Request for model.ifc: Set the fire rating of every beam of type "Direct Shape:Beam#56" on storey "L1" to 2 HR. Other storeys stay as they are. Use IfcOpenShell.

First a look at what the model holds.

```python
import ifcopenshell
import ifcopenshell.util.element

model = ifcopenshell.open("model.ifc")
print(model.schema)
storey = next(s for s in model.by_type("IfcBuildingStorey") if s.Name == "L1")
beams = [e for e in ifcopenshell.util.element.get_decomposition(storey) if e.is_a("IfcBeam")]
seen = {}
for e in beams:
    element_type = ifcopenshell.util.element.get_type(e)
    key = (element_type.Name if element_type != e and element_type else None, ifcopenshell.util.element.get_pset(e, "Pset_BeamCommon", "FireRating"))
    seen[key] = seen.get(key, 0) + 1
for (name, value), count in sorted(seen.items(), key=str):
    print(count, "x", name, "|", value)
```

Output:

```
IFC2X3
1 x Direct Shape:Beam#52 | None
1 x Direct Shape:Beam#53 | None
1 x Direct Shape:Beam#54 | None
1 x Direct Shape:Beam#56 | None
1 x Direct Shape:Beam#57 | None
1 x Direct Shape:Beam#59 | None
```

```python
import ifcopenshell
import ifcopenshell.api.pset
import ifcopenshell.util.element

model = ifcopenshell.open("model.ifc")

storey = next(s for s in model.by_type("IfcBuildingStorey") if s.Name == "L1")
beams = [e for e in ifcopenshell.util.element.get_decomposition(storey) if e.is_a("IfcBeam")]

count = 0
for e in beams:
    element_type = ifcopenshell.util.element.get_type(e)
    if element_type in (None, e) or element_type.Name != "Direct Shape:Beam#56":
        continue
    # add_pset returns the element's existing set when there is one.
    pset = ifcopenshell.api.pset.add_pset(model, product=e, name="Pset_BeamCommon")
    ifcopenshell.api.pset.edit_pset(model, pset=pset, properties={"FireRating": "2 HR"})
    count += 1

print(count, "beams updated")

model.write("model_edited.ifc")
```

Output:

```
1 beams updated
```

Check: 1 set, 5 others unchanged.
